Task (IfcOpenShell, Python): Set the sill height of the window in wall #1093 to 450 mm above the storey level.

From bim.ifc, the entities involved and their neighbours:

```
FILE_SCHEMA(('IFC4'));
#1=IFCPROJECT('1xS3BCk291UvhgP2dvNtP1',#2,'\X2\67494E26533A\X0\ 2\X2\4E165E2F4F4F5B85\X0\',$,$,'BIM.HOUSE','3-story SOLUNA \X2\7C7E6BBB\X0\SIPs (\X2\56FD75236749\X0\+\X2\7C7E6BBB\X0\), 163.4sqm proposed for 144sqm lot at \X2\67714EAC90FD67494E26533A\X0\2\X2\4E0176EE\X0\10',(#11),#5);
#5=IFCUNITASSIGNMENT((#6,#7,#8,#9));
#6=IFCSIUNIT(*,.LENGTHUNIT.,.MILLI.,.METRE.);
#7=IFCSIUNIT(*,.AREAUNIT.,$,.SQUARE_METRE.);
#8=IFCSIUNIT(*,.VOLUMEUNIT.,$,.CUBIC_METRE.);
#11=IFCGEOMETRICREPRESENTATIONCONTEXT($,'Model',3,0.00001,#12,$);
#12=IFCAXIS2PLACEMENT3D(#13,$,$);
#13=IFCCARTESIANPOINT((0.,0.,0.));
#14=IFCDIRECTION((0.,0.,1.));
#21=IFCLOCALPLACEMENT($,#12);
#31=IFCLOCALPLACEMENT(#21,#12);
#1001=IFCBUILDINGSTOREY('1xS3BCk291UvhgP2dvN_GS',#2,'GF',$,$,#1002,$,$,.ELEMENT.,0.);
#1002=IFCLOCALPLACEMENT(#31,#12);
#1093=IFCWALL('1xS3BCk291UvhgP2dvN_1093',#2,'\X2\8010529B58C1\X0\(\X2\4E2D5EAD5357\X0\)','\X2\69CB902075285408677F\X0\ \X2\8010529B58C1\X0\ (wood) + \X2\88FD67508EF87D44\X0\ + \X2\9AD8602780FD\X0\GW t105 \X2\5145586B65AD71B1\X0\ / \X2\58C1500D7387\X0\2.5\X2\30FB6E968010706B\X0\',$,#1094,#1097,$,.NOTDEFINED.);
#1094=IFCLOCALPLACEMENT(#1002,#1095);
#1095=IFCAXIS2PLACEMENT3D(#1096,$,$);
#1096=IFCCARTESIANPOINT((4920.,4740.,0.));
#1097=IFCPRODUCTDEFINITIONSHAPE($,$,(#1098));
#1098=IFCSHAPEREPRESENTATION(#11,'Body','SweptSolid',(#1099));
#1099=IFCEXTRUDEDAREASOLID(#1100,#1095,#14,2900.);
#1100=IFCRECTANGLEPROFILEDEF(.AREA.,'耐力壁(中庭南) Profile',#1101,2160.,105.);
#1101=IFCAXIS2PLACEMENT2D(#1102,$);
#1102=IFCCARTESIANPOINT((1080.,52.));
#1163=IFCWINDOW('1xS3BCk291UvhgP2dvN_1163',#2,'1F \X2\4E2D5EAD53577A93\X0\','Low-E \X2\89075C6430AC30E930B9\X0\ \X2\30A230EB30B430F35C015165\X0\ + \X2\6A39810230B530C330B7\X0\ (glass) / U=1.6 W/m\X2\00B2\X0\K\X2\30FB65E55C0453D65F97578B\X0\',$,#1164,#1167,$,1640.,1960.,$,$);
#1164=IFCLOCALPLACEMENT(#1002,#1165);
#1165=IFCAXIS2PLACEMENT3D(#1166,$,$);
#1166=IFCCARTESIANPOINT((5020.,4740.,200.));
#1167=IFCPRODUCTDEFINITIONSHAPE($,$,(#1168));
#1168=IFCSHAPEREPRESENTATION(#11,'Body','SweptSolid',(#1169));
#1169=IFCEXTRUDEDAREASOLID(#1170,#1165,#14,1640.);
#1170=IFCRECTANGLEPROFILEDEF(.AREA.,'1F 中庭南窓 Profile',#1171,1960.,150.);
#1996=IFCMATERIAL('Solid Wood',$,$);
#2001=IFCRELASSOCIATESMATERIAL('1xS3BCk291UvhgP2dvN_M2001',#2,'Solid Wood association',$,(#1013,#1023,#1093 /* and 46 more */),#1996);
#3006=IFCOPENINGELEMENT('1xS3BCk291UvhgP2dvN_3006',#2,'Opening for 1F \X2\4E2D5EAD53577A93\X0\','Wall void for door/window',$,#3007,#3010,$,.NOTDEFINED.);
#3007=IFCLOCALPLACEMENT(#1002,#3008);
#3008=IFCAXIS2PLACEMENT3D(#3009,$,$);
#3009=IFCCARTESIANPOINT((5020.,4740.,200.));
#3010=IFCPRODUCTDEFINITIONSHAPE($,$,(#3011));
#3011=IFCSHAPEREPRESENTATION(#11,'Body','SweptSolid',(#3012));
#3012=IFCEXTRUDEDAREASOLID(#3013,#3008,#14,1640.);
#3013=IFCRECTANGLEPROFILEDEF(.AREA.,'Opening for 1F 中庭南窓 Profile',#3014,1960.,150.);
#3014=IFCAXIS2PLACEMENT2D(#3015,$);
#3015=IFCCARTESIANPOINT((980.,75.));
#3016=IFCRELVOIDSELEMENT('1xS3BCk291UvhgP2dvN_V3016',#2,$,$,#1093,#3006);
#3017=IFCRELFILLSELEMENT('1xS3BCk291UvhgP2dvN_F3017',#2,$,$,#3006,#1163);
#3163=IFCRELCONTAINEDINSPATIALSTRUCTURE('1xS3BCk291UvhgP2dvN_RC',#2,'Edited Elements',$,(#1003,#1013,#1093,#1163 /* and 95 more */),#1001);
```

```python
import numpy as np
import ifcopenshell
import ifcopenshell.api.geometry
import ifcopenshell.geom
import ifcopenshell.util.element
import ifcopenshell.util.placement
import ifcopenshell.util.shape
import ifcopenshell.util.unit

model = ifcopenshell.open("bim.ifc")
unit_scale = ifcopenshell.util.unit.calculate_unit_scale(model)

window = model.by_guid("1xS3BCk291UvhgP2dvN_1163")
opening = window.FillsVoids[0].RelatingOpeningElement
storey = ifcopenshell.util.element.get_container(window, ifc_class="IfcBuildingStorey")
level = ifcopenshell.util.placement.get_local_placement(storey.ObjectPlacement)[2, 3]

# The opening's origin need not be at the sill, so measure its lowest point.
shape = ifcopenshell.geom.create_shape(ifcopenshell.geom.settings(), opening)
bottom = ifcopenshell.util.shape.get_shape_bottom_elevation(shape, shape.geometry) / unit_scale
dz = level + 450.0 - bottom

shift = np.array([0.0, 0.0, dz])
# The window is not placed relative to its opening, so move both.
for product in (opening, window):
    matrix = ifcopenshell.util.placement.get_local_placement(product.ObjectPlacement)
    matrix[:3, 3] += shift
    ifcopenshell.api.geometry.edit_object_placement(model, product=product, matrix=matrix, is_si=False)

print(f"moved by {dz * unit_scale:+.3f} m")

model.write("bim-out.ifc")
```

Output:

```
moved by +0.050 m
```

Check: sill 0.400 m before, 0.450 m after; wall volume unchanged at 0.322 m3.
